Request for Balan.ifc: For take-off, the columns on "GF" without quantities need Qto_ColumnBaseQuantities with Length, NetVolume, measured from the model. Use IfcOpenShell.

First a look at what the model holds.

```python
import ifcopenshell
import ifcopenshell.util.element
import ifcopenshell.util.unit

model = ifcopenshell.open("Balan.ifc")
print(model.schema)
for unit_type in ("LENGTHUNIT", "AREAUNIT", "VOLUMEUNIT"):
    print(unit_type, ifcopenshell.util.unit.calculate_unit_scale(model, unit_type))
storey = next(s for s in model.by_type("IfcBuildingStorey") if s.Name == "GF")
columns = [e for e in ifcopenshell.util.element.get_decomposition(storey) if e.is_a("IfcColumn")]
for e in sorted(columns, key=lambda e: e.id()):
    print(e.id(), e.is_a(), e.Name, list(ifcopenshell.util.element.get_psets(e, qtos_only=True)), sep=" | ")
```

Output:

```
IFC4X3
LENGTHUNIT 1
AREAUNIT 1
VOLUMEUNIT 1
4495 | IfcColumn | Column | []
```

```python
import ifcopenshell
import ifcopenshell.api.pset
import ifcopenshell.geom
import ifcopenshell.util.element
import ifcopenshell.util.shape
import ifcopenshell.util.unit

model = ifcopenshell.open("Balan.ifc")
unit_scale = ifcopenshell.util.unit.calculate_unit_scale(model)
volume_scale = ifcopenshell.util.unit.calculate_unit_scale(model, "VOLUMEUNIT")
settings = ifcopenshell.geom.settings()

storey = next(s for s in model.by_type("IfcBuildingStorey") if s.Name == "GF")
columns = [e for e in ifcopenshell.util.element.get_decomposition(storey) if e.is_a("IfcColumn")]

for e in sorted(columns, key=lambda e: e.id()):
    if ifcopenshell.util.element.get_psets(e, qtos_only=True, should_inherit=False):
        continue
    # Geometry comes back in metres, in the element's own axes.
    shape = ifcopenshell.geom.create_shape(settings, e)
    values = {
        "Length": ifcopenshell.util.shape.get_z(shape.geometry) / unit_scale,
        "NetVolume": ifcopenshell.util.shape.get_volume(shape.geometry) / volume_scale,
    }
    qto = ifcopenshell.api.pset.add_qto(model, product=e, name="Qto_ColumnBaseQuantities")
    ifcopenshell.api.pset.edit_qto(model, qto=qto, properties=values)
    print(e.id(), {k: round(v, 3) for k, v in values.items()})

model.write("Balan-out.ifc")
```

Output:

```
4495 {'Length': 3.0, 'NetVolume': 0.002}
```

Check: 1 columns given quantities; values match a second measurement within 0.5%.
